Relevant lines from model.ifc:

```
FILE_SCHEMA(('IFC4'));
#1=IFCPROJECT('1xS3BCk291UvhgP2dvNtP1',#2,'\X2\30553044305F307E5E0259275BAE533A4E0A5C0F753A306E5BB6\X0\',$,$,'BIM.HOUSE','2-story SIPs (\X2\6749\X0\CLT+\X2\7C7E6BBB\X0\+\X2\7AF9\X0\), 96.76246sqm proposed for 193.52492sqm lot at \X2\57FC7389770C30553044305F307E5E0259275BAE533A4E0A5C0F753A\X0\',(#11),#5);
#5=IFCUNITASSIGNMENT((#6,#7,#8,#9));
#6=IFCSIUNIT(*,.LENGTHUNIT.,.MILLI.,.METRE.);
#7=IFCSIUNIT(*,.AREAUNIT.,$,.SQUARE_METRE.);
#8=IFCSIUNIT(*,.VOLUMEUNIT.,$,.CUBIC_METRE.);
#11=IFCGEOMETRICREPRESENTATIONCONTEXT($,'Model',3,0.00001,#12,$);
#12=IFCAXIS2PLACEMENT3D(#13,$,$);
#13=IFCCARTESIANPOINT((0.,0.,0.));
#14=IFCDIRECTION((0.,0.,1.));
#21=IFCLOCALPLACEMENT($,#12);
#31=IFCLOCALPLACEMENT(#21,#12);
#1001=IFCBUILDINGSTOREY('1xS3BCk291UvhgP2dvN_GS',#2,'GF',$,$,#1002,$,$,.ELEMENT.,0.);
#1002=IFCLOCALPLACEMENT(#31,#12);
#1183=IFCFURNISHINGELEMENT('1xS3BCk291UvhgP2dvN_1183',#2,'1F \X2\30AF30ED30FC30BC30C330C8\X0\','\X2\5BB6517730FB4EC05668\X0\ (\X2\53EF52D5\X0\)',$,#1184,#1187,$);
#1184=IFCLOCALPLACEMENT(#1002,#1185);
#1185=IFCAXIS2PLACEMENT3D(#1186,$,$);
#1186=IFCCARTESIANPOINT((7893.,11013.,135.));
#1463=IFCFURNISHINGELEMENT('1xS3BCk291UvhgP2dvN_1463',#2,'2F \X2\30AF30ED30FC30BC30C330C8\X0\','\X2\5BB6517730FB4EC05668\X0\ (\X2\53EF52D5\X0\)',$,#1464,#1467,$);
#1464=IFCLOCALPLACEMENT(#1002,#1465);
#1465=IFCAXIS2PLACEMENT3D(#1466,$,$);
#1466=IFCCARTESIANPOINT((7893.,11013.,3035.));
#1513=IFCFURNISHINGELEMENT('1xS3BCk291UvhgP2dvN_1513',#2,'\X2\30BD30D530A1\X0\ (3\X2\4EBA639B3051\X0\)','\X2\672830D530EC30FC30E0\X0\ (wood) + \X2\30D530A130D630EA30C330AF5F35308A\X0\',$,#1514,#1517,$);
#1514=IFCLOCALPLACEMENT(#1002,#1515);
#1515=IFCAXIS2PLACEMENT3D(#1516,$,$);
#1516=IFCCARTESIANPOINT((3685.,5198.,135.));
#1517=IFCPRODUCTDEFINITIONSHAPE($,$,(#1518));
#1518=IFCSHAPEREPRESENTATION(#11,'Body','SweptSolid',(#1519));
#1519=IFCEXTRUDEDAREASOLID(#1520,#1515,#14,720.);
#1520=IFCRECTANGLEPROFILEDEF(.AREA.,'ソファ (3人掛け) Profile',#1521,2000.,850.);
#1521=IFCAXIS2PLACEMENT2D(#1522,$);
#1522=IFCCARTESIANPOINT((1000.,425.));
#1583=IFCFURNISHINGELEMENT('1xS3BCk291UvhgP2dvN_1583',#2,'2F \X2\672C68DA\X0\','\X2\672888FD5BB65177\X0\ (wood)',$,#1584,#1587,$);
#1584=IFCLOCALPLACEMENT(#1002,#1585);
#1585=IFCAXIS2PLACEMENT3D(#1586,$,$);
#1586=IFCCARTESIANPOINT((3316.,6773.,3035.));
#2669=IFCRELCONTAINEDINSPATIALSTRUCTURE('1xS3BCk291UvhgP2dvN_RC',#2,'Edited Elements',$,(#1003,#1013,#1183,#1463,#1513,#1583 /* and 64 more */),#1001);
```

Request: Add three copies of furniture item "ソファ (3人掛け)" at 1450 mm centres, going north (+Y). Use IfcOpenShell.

```python
import numpy as np
import ifcopenshell
import ifcopenshell.api.geometry
import ifcopenshell.api.root
import ifcopenshell.util.element
import ifcopenshell.util.placement
import ifcopenshell.util.unit

model = ifcopenshell.open("model.ifc")
unit_scale = ifcopenshell.util.unit.calculate_unit_scale(model)


def reuse_history(source, copy):
    """copy_class also copies each property set's owner history, people and application; keep the originals."""
    for rel in copy.IsDefinedBy:
        if rel.is_a("IfcRelDefinesByProperties") and (history := rel.RelatingPropertyDefinition.OwnerHistory):
            rel.RelatingPropertyDefinition.OwnerHistory = source.OwnerHistory
            ifcopenshell.util.element.remove_deep2(model, history)


source = model.by_guid("1xS3BCk291UvhgP2dvN_1513")
base = ifcopenshell.util.placement.get_local_placement(source.ObjectPlacement)
step = np.array([0.0, 1.0, 0.0]) * 1.45 / unit_scale

for i in range(1, 4):
    copy = ifcopenshell.api.root.copy_class(model, product=source)
    copy.Representation = ifcopenshell.util.element.copy_deep(
        model, source.Representation, exclude=["IfcGeometricRepresentationContext", "IfcRepresentationMap"]
    )
    reuse_history(source, copy)
    matrix = base.copy()
    matrix[:3, 3] += i * step
    print("added at", matrix[:3, 3].round(3) + 0.0)
    ifcopenshell.api.geometry.edit_object_placement(model, product=copy, matrix=matrix, is_si=False)

model.write("model-out.ifc")
```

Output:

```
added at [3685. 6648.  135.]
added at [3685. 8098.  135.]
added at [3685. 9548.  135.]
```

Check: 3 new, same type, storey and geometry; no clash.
